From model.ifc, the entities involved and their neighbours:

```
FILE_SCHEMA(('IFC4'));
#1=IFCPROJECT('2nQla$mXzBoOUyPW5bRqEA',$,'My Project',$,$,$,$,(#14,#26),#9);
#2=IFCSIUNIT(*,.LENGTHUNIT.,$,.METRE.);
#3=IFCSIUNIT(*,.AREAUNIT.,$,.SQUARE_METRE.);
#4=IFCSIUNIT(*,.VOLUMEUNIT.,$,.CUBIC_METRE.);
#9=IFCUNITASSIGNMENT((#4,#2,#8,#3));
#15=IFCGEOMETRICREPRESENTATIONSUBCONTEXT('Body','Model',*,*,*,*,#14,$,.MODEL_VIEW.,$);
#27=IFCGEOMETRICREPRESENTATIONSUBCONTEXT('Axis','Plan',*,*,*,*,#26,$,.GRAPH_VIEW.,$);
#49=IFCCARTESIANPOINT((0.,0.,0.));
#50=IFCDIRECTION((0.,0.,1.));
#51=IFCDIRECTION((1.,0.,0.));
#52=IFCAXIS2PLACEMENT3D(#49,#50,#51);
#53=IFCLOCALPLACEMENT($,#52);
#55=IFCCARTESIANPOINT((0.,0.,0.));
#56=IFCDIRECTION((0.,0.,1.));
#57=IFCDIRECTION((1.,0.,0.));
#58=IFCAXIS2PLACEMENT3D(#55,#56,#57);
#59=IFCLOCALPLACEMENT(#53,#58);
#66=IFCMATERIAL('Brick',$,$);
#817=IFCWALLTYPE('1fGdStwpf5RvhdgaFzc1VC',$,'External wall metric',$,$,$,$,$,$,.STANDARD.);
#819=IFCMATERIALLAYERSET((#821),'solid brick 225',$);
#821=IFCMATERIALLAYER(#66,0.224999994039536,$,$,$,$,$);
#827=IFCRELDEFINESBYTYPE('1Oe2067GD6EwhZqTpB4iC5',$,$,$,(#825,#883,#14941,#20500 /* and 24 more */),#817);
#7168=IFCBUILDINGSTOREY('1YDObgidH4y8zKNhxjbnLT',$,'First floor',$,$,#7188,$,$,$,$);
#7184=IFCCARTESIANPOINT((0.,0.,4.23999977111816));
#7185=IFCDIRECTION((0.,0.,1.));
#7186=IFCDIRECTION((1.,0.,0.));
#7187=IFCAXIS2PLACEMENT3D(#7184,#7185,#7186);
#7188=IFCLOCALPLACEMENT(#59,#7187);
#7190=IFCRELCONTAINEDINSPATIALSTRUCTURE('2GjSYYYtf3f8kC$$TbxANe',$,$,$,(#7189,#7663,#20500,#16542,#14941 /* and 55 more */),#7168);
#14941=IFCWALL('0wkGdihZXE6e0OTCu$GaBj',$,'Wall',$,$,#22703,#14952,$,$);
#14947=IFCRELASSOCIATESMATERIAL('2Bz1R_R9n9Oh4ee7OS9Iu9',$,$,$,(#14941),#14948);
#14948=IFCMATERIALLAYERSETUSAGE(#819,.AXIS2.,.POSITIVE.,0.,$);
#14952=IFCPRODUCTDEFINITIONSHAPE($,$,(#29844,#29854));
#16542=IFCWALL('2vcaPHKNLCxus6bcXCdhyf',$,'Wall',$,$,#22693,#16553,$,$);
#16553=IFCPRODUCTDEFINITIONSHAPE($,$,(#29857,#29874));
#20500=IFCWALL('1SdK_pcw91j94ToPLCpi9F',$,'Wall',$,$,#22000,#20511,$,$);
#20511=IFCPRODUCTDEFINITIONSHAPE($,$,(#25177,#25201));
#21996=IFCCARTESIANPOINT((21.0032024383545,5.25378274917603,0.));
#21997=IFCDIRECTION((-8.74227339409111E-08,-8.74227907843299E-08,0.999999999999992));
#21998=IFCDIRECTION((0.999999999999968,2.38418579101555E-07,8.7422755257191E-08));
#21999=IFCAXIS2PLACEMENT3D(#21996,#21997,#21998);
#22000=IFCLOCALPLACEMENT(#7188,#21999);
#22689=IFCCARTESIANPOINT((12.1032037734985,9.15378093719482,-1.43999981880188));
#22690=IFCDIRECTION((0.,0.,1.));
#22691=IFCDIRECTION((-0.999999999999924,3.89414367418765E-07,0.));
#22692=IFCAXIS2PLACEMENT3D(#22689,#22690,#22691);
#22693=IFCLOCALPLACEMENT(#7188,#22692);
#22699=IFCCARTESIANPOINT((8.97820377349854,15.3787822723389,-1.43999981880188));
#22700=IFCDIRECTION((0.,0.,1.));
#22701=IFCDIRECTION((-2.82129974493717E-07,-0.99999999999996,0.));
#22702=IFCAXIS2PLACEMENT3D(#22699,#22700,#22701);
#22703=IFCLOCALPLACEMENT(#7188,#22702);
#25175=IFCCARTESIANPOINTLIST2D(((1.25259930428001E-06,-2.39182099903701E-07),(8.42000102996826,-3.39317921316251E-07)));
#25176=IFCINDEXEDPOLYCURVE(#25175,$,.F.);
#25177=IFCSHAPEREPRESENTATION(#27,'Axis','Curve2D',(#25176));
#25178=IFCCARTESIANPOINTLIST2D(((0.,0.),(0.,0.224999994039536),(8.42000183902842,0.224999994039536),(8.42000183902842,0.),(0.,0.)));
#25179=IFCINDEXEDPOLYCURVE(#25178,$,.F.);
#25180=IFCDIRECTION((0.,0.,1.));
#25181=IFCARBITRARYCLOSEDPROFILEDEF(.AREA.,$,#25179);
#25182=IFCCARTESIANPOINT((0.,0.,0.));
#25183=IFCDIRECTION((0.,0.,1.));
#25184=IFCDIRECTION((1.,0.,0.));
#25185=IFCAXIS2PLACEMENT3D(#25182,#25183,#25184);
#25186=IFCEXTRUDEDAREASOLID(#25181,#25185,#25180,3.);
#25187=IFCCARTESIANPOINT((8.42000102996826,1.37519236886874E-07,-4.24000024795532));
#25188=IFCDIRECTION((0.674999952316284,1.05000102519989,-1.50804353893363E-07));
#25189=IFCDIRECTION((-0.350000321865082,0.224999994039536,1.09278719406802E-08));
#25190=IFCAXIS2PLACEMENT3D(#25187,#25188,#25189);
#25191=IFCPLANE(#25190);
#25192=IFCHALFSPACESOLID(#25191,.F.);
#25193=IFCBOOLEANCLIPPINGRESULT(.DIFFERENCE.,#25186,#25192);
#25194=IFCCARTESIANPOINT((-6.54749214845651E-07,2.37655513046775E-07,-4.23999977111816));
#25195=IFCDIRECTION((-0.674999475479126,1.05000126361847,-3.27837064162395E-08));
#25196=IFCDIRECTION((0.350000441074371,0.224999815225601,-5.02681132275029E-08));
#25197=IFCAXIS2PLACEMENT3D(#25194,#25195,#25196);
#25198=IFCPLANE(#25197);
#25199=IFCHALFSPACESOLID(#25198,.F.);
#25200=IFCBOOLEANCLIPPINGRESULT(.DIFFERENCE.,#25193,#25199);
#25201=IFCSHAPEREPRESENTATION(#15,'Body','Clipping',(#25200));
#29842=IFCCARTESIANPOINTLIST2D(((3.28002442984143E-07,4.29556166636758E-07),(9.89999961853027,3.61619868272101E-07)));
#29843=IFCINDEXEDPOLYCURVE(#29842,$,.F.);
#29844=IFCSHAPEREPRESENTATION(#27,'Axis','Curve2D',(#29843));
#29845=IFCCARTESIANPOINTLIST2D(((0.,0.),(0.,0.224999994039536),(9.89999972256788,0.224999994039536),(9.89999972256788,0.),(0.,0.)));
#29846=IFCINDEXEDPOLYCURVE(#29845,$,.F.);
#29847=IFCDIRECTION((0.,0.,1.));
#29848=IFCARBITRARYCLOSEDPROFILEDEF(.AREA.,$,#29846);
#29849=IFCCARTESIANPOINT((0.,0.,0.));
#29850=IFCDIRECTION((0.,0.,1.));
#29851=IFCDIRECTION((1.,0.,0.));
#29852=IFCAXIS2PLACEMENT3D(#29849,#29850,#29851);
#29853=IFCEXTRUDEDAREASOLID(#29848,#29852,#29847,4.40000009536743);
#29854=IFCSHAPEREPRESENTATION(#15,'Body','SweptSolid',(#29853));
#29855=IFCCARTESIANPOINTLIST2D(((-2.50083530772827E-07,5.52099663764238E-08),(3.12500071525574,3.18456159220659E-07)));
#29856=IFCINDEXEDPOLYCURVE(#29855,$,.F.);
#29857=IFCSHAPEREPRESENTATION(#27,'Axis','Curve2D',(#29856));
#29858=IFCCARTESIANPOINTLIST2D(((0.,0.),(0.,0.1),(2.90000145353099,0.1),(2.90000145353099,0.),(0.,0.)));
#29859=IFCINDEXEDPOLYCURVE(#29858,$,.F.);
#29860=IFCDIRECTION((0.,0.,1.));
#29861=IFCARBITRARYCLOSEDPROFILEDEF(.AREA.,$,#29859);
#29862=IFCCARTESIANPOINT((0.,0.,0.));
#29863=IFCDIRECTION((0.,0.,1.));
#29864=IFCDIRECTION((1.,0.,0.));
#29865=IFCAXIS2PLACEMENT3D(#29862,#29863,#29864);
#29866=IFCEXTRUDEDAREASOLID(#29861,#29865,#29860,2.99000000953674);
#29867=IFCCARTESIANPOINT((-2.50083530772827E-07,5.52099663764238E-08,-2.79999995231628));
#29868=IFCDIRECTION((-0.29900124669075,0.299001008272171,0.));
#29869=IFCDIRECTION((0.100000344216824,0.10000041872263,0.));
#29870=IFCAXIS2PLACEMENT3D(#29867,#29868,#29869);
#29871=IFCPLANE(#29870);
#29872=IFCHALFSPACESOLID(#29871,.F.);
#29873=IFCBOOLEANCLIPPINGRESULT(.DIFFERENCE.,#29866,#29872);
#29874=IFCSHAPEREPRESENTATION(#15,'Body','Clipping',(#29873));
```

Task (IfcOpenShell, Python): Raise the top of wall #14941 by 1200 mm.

```python
import ifcopenshell
import ifcopenshell.geom
import ifcopenshell.util.representation
import ifcopenshell.util.shape

model = ifcopenshell.open("model.ifc")
settings = ifcopenshell.geom.settings()


def volume(element):
    """Net volume in cubic metres, openings subtracted."""
    shape = ifcopenshell.geom.create_shape(settings, element)
    return ifcopenshell.util.shape.get_volume(shape.geometry)


wall = model.by_guid("0wkGdihZXE6e0OTCu$GaBj")
before = volume(wall)

body = ifcopenshell.util.representation.get_representation(wall, "Model", "Body")
solid = body.Items[0]
old_height = solid.Depth
solid.Depth += 1.2
after = volume(wall)

print(f"height {old_height:g} -> {solid.Depth:g}, volume {before:.3f} -> {after:.3f} m3")

model.write("model_edited.ifc")
```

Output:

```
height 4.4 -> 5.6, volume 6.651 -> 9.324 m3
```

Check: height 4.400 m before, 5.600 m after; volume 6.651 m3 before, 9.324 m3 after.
